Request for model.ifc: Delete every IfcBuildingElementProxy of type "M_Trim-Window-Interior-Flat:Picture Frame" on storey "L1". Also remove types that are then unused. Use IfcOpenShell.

First a look at what the model holds.

```python
import ifcopenshell
import ifcopenshell.util.element

model = ifcopenshell.open("model.ifc")
print(model.schema)
storey = next(s for s in model.by_type("IfcBuildingStorey") if s.Name == "L1")
proxies = [e for e in ifcopenshell.util.element.get_decomposition(storey) if e.is_a("IfcBuildingElementProxy")]
seen = {}
for e in proxies:
    element_type = ifcopenshell.util.element.get_type(e)
    name = element_type.Name if element_type not in (None, e) else None
    seen[name] = seen.get(name, 0) + 1
for name, count in sorted(seen.items(), key=str):
    print(count, "x", name)
```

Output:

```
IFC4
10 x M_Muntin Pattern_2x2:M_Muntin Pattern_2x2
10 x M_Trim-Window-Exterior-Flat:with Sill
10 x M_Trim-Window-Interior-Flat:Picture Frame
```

```python
import ifcopenshell
import ifcopenshell.api.root
import ifcopenshell.util.element

model = ifcopenshell.open("model.ifc")

storey = next(s for s in model.by_type("IfcBuildingStorey") if s.Name == "L1")
proxies = [e for e in ifcopenshell.util.element.get_decomposition(storey) if e.is_a("IfcBuildingElementProxy")]
targets = [e for e in proxies if (t := ifcopenshell.util.element.get_type(e)) not in (None, e) and t.Name == "M_Trim-Window-Interior-Flat:Picture Frame"]
types = {ifcopenshell.util.element.get_type(e) for e in targets} - {None, *targets}

for e in targets:
    ifcopenshell.api.root.remove_product(model, product=e)
print(len(targets), "removed")

unused = [t for t in types if not ifcopenshell.util.element.get_types(t)]
for t in unused:
    ifcopenshell.api.root.remove_product(model, product=t)
print(len(unused), "unused types removed")

model.write("model_rev.ifc")
```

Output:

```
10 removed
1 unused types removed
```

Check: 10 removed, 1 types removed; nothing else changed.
